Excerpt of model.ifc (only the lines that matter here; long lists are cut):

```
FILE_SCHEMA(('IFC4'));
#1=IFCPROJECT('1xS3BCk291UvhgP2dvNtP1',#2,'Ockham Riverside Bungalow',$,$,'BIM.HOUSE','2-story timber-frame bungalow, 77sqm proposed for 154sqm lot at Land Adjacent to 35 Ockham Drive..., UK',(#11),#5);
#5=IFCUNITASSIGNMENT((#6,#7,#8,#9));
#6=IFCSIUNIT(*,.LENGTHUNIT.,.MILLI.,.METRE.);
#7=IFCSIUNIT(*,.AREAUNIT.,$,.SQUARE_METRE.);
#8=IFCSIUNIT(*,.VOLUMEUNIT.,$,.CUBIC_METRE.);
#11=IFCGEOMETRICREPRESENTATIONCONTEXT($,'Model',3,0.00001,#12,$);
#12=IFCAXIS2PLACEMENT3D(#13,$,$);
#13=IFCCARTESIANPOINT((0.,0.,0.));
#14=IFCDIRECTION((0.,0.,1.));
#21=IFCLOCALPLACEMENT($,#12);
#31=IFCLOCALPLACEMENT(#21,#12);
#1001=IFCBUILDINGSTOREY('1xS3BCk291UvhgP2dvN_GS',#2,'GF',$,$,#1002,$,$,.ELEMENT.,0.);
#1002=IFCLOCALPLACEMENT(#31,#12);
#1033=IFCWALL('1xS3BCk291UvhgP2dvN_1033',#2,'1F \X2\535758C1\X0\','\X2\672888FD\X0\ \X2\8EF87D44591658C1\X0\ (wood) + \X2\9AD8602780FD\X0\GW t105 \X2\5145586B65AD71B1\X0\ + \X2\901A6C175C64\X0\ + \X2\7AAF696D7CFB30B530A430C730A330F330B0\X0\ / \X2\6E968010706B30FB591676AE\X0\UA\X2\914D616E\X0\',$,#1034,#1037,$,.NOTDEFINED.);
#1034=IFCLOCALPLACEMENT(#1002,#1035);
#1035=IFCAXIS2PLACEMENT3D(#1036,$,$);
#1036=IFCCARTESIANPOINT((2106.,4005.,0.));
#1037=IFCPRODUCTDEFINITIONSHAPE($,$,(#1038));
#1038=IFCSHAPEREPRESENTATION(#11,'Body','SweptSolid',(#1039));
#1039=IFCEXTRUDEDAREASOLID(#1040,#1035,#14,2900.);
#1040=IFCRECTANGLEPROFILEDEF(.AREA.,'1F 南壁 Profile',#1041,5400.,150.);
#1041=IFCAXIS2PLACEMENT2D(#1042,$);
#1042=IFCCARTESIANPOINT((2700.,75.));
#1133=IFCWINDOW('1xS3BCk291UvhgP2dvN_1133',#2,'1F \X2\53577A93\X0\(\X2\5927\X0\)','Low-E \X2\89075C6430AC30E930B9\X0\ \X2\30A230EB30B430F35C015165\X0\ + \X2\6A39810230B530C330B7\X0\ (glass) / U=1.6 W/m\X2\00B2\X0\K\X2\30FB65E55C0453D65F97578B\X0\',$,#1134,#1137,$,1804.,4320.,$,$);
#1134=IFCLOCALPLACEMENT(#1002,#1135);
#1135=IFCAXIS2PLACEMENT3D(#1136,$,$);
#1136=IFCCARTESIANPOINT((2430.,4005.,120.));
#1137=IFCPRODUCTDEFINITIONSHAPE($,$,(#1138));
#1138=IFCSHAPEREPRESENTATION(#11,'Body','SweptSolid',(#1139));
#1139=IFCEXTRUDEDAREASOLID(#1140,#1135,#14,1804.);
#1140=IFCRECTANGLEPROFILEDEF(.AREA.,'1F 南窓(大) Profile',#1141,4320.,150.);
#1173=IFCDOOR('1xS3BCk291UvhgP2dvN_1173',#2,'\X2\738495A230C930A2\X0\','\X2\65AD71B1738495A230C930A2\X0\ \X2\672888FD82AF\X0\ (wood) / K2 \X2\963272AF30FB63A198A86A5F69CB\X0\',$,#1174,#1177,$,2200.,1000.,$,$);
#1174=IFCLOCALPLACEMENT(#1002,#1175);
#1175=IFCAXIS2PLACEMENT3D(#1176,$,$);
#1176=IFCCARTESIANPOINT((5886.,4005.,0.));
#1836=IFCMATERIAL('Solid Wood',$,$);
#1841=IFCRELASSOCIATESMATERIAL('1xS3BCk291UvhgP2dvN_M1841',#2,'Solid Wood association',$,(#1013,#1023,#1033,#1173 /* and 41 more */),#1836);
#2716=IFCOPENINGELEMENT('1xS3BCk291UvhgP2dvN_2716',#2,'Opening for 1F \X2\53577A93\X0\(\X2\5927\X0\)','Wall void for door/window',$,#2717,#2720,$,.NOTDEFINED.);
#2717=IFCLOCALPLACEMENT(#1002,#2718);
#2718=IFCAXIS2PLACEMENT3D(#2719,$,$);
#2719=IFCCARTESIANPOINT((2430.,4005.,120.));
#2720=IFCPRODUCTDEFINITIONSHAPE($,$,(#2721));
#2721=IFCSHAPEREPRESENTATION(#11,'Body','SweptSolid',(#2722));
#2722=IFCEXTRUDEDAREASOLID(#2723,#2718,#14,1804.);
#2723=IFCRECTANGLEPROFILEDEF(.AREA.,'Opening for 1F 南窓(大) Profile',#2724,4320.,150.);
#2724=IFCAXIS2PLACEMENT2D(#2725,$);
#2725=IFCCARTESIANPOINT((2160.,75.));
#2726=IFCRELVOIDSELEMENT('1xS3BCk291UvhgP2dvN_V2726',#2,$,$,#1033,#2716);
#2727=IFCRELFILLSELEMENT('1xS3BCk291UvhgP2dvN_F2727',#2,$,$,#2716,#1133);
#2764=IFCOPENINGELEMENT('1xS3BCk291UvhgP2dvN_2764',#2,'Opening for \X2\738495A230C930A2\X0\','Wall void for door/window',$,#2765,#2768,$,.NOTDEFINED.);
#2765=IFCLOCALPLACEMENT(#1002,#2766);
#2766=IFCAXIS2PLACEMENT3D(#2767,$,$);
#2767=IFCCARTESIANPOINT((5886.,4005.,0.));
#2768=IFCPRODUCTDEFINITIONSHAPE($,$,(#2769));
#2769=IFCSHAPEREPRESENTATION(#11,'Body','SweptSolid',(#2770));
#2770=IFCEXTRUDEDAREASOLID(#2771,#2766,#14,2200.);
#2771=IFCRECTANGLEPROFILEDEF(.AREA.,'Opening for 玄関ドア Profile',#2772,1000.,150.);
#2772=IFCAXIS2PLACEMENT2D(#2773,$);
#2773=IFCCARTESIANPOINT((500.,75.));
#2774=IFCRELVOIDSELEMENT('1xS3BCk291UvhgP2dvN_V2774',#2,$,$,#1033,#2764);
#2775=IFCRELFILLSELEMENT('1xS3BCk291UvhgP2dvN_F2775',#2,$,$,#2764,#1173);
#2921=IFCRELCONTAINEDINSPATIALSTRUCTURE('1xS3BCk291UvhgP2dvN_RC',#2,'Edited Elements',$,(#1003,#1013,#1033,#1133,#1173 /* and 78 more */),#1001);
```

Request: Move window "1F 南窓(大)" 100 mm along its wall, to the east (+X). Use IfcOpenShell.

```python
import ifcopenshell
import ifcopenshell.api.geometry
import ifcopenshell.util.placement

model = ifcopenshell.open("model.ifc")

window = model.by_guid("1xS3BCk291UvhgP2dvN_1133")
opening = window.FillsVoids[0].RelatingOpeningElement
wall = opening.VoidsElements[0].RelatingBuildingElement

wall_matrix = ifcopenshell.util.placement.get_local_placement(wall.ObjectPlacement)
shift = wall_matrix[:3, 0] * 100.0
before = ifcopenshell.util.placement.get_local_placement(window.ObjectPlacement)[:3, 3].copy()

# The window is not placed relative to its opening, so move both.
for product in (opening, window):
    matrix = ifcopenshell.util.placement.get_local_placement(product.ObjectPlacement)
    matrix[:3, 3] += shift
    ifcopenshell.api.geometry.edit_object_placement(model, product=product, matrix=matrix, is_si=False)

after = ifcopenshell.util.placement.get_local_placement(window.ObjectPlacement)[:3, 3]
print("window moved by", (after - before).round(3) + 0.0)

model.write("model_rev.ifc")
```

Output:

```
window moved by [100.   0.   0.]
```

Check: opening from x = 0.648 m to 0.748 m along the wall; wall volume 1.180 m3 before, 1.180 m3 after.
